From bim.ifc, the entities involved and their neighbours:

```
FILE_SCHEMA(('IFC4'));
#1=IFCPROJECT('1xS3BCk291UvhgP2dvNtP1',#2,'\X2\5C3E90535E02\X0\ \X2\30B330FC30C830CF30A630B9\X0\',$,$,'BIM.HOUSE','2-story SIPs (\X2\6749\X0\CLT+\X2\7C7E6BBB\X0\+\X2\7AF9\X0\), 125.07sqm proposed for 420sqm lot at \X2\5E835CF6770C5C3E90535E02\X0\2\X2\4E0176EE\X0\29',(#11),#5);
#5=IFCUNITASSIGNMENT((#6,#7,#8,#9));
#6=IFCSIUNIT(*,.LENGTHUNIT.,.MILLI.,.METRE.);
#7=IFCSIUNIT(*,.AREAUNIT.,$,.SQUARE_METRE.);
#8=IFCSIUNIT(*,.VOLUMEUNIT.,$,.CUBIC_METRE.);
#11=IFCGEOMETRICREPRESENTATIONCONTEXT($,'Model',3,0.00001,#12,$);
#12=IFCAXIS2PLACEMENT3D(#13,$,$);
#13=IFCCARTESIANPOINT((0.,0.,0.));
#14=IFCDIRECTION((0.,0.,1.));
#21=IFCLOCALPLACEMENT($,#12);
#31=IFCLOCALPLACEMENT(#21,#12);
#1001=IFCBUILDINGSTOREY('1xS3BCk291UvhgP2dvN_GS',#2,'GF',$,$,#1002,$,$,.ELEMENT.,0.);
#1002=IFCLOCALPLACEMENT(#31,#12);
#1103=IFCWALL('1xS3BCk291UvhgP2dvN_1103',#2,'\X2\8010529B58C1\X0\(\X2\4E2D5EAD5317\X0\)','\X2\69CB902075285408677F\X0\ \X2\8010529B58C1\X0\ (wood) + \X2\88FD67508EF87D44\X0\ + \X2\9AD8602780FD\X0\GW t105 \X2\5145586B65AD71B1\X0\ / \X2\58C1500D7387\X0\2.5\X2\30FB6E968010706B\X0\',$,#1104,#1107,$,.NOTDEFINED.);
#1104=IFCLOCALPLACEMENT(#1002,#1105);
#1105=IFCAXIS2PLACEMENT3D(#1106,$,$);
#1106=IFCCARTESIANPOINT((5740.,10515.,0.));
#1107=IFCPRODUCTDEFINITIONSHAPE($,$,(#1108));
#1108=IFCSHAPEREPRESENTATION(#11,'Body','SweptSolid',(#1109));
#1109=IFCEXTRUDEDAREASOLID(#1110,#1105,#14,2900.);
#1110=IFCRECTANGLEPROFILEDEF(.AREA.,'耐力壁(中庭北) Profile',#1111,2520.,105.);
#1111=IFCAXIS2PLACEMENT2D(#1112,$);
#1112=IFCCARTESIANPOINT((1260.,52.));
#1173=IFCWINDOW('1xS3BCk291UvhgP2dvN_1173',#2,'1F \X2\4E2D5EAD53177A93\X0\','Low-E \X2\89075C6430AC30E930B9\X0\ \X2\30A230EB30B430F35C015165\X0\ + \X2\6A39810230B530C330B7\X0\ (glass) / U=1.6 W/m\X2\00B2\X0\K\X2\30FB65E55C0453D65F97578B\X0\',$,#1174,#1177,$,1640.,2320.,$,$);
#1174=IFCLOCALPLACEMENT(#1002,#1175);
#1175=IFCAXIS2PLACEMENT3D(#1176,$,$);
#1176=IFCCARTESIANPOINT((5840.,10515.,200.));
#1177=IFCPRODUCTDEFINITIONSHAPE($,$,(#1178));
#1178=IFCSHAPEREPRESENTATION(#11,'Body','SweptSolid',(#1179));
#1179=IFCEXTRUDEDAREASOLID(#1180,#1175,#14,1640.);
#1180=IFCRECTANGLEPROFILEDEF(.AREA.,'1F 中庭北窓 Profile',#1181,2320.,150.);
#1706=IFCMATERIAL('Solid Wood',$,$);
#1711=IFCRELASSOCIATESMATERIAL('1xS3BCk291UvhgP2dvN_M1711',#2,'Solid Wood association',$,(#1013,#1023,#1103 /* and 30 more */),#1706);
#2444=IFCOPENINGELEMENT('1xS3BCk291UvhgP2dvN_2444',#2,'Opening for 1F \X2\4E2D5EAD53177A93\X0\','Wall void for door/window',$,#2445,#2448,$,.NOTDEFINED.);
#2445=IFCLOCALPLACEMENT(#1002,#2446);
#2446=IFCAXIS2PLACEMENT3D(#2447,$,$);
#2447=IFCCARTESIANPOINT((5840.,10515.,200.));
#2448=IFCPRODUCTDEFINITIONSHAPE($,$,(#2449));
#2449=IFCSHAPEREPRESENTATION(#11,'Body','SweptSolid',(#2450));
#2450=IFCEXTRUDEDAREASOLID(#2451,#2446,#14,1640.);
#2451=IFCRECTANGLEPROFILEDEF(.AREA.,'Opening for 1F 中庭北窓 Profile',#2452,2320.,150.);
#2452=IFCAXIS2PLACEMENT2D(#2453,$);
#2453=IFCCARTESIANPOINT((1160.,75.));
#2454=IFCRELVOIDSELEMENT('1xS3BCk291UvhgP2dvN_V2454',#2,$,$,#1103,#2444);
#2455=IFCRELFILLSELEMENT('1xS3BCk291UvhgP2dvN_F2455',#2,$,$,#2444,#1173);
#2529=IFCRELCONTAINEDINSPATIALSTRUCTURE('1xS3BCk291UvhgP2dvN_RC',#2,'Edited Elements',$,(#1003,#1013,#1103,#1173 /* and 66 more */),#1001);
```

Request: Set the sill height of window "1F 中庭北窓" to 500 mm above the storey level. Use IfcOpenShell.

```python
import numpy as np
import ifcopenshell
import ifcopenshell.api.geometry
import ifcopenshell.geom
import ifcopenshell.util.element
import ifcopenshell.util.placement
import ifcopenshell.util.shape
import ifcopenshell.util.unit

model = ifcopenshell.open("bim.ifc")
unit_scale = ifcopenshell.util.unit.calculate_unit_scale(model)

window = model.by_guid("1xS3BCk291UvhgP2dvN_1173")
opening = window.FillsVoids[0].RelatingOpeningElement
storey = ifcopenshell.util.element.get_container(window, ifc_class="IfcBuildingStorey")
level = ifcopenshell.util.placement.get_local_placement(storey.ObjectPlacement)[2, 3]

# The opening's origin need not be at the sill, so measure its lowest point.
shape = ifcopenshell.geom.create_shape(ifcopenshell.geom.settings(), opening)
bottom = ifcopenshell.util.shape.get_shape_bottom_elevation(shape, shape.geometry) / unit_scale
dz = level + 500.0 - bottom

shift = np.array([0.0, 0.0, dz])
# The window is not placed relative to its opening, so move both.
for product in (opening, window):
    matrix = ifcopenshell.util.placement.get_local_placement(product.ObjectPlacement)
    matrix[:3, 3] += shift
    ifcopenshell.api.geometry.edit_object_placement(model, product=product, matrix=matrix, is_si=False)

print(f"moved by {dz * unit_scale:+.3f} m")

model.write("bim_edited.ifc")
```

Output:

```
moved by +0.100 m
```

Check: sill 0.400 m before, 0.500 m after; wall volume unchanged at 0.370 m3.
